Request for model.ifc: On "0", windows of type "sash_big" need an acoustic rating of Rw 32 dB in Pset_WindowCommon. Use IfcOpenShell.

First a look at what the model holds.

```python
import ifcopenshell
import ifcopenshell.util.element

model = ifcopenshell.open("model.ifc")
print(model.schema)
storey = next(s for s in model.by_type("IfcBuildingStorey") if s.Name == "0")
windows = [e for e in ifcopenshell.util.element.get_decomposition(storey) if e.is_a("IfcWindow")]
seen = {}
for e in windows:
    element_type = ifcopenshell.util.element.get_type(e)
    key = (element_type.Name if element_type != e and element_type else None, ifcopenshell.util.element.get_pset(e, "Pset_WindowCommon", "AcousticRating"))
    seen[key] = seen.get(key, 0) + 1
for (name, value), count in sorted(seen.items(), key=str):
    print(count, "x", name, "|", value)
```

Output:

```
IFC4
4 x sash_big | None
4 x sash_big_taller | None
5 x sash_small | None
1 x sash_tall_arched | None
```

```python
import ifcopenshell
import ifcopenshell.api.pset
import ifcopenshell.util.element

model = ifcopenshell.open("model.ifc")

storey = next(s for s in model.by_type("IfcBuildingStorey") if s.Name == "0")
windows = [e for e in ifcopenshell.util.element.get_decomposition(storey) if e.is_a("IfcWindow")]

count = 0
for e in windows:
    element_type = ifcopenshell.util.element.get_type(e)
    if element_type in (None, e) or element_type.Name != "sash_big":
        continue
    # add_pset returns the element's existing set when there is one.
    pset = ifcopenshell.api.pset.add_pset(model, product=e, name="Pset_WindowCommon")
    ifcopenshell.api.pset.edit_pset(model, pset=pset, properties={"AcousticRating": "Rw 32 dB"})
    count += 1

print(count, "windows updated")

model.write("model_rev.ifc")
```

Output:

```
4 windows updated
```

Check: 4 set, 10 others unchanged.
